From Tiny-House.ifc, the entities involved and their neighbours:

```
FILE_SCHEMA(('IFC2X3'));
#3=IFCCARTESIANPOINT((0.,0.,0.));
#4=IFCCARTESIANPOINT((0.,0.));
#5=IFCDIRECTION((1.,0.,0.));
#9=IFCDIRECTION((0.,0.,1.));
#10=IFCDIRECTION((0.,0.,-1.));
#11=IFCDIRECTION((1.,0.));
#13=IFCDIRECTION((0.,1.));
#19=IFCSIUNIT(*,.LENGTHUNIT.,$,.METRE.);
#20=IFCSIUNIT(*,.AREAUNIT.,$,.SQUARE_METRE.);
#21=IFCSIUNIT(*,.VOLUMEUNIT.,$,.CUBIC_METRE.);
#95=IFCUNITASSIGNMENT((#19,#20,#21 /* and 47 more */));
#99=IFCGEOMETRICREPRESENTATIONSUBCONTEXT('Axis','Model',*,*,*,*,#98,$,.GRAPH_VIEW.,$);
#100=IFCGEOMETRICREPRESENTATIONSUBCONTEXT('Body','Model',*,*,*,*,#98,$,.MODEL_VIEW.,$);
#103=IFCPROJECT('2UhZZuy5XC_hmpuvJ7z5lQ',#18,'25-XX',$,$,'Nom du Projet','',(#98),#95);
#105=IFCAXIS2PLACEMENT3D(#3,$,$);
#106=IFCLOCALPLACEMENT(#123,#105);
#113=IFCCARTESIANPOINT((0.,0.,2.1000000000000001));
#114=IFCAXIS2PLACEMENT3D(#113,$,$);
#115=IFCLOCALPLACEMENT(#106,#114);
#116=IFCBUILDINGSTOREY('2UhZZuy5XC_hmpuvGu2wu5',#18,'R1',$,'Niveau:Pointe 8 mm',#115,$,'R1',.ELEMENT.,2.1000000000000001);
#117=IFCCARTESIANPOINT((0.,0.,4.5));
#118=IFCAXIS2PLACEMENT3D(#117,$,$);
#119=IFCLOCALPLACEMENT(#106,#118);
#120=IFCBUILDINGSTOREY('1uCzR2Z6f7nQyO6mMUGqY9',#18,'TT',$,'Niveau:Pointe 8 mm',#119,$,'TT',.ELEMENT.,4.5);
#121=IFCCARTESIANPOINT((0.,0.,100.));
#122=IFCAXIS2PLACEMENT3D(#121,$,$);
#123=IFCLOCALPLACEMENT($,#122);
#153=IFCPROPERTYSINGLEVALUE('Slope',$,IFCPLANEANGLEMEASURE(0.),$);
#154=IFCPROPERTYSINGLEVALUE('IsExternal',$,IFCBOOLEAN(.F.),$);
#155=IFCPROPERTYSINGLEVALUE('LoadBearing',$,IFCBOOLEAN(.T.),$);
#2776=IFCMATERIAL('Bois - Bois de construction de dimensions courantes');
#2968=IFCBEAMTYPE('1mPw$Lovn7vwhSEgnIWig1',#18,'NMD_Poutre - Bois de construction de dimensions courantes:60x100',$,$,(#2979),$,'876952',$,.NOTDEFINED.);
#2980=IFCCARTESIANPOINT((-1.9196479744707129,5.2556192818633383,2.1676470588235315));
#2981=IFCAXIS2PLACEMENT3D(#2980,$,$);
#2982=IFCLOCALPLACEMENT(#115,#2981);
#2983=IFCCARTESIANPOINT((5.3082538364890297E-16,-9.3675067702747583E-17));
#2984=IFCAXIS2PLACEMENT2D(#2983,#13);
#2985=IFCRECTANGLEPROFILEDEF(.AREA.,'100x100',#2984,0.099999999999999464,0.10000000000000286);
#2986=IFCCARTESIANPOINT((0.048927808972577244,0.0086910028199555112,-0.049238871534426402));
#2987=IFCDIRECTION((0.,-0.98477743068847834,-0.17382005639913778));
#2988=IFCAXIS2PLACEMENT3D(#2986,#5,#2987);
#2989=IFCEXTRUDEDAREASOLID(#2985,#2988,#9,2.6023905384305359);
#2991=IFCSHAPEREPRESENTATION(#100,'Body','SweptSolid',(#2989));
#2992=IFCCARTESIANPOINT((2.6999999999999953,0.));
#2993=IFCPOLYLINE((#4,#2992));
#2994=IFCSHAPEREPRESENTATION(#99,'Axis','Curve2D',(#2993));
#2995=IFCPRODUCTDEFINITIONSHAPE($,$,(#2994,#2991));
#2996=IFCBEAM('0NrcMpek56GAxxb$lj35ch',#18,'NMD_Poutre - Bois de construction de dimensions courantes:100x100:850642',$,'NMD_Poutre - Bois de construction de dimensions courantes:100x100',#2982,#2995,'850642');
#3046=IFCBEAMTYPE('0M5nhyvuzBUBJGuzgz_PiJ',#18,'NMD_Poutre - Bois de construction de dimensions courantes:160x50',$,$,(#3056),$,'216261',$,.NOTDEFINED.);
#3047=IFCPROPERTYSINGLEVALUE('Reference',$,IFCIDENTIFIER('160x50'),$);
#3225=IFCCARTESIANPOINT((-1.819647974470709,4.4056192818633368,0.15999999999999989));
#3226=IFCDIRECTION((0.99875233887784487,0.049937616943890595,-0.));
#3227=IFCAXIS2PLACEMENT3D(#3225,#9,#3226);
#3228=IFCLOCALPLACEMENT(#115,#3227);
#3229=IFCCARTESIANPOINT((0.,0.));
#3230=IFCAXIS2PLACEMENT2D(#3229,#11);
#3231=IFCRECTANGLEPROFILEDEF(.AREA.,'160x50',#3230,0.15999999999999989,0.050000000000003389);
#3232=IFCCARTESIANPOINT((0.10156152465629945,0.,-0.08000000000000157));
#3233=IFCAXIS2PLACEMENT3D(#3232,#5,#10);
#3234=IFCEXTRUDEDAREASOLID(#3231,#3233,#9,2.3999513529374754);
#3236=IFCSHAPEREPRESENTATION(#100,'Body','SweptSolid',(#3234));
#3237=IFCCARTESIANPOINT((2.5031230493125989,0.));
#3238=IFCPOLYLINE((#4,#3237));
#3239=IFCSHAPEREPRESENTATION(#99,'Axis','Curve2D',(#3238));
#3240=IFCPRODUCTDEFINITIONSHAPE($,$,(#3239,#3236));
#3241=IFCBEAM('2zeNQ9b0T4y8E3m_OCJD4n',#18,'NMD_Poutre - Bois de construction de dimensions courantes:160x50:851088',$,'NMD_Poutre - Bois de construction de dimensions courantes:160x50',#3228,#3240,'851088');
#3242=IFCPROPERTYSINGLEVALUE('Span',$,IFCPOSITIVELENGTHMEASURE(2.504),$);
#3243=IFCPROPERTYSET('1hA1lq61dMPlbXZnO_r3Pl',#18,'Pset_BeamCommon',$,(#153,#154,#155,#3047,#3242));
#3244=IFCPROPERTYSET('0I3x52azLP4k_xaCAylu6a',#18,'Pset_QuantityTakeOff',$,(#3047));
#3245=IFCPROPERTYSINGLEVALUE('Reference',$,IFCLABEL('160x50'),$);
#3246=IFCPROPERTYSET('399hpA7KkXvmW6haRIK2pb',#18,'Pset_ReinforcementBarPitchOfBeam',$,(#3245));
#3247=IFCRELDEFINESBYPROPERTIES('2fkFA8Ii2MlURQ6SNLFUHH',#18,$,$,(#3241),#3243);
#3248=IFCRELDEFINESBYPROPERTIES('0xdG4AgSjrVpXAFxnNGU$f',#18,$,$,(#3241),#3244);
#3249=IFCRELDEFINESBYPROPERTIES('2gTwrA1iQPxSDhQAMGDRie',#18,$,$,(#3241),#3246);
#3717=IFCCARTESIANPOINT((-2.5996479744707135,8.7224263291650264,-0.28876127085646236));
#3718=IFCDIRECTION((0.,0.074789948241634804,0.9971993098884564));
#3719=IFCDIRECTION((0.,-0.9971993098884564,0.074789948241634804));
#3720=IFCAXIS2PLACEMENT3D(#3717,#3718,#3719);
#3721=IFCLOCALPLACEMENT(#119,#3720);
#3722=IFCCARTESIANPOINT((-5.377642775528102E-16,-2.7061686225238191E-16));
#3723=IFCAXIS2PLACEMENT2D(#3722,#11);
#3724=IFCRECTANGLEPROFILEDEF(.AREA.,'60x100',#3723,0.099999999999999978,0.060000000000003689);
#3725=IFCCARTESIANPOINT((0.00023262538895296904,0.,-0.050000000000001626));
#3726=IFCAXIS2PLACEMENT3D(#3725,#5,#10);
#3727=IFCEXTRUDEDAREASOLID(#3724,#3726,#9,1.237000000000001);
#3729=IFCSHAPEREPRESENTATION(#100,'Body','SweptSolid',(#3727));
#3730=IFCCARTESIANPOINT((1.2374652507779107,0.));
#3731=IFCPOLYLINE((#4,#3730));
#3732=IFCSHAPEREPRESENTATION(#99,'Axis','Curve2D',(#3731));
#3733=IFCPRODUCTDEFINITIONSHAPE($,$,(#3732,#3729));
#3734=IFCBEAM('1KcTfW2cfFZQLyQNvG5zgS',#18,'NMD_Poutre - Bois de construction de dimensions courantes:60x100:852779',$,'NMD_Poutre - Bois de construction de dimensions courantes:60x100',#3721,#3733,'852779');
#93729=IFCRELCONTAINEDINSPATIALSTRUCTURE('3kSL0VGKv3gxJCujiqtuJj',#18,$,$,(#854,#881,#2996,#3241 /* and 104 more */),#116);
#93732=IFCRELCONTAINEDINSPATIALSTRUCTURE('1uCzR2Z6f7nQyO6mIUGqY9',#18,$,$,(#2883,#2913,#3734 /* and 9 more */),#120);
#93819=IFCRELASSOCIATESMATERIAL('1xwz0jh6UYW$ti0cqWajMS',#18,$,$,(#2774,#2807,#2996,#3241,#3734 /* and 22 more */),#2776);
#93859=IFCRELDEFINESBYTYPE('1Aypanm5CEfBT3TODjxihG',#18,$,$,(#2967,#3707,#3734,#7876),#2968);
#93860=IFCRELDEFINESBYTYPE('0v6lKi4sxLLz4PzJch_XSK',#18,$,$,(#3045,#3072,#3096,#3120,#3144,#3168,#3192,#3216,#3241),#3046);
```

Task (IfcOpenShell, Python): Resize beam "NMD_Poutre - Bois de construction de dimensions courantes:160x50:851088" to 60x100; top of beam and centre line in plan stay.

```python
import ifcopenshell
import ifcopenshell.api.pset
import ifcopenshell.api.type
import ifcopenshell.util.element
import ifcopenshell.util.representation

model = ifcopenshell.open("Tiny-House.ifc")

member = model.by_guid("2zeNQ9b0T4y8E3m_OCJD4n")
source = next(p for p in model.by_type("IfcRectangleProfileDef") if p.ProfileName == "60x100")

body = ifcopenshell.util.representation.get_representation(member, "Model", "Body")
solid = body.Items[0]
old_profile = solid.SweptArea

# Copy the section's sizes but keep this member's own profile position.
profile = ifcopenshell.util.element.copy(model, source)
# Profiles are centred, so shift by half the change in depth to hold the top.
shift = (old_profile.XDim - profile.XDim) / 2
x, y = old_profile.Position.Location.Coordinates
up = (-1.0, 0.0)  # upwards, in the solid's own plane
location = model.createIfcCartesianPoint((x + up[0] * shift, y + up[1] * shift))
profile.Position = model.createIfcAxis2Placement2D(location, old_profile.Position.RefDirection)
solid.SweptArea = profile
if not model.get_total_inverses(old_profile):
    ifcopenshell.util.element.remove_deep2(model, old_profile)

new_type = model.by_guid("1mPw$Lovn7vwhSEgnIWig1")
ifcopenshell.api.type.assign_type(
    model, related_objects=[member], relating_type=new_type, should_map_representations=False
)
member.Name = member.Name.replace("160x50", "60x100")
member.ObjectType = "NMD_Poutre - Bois de construction de dimensions courantes:60x100"
pset = model.by_id(ifcopenshell.util.element.get_pset(member, "Pset_BeamCommon", should_inherit=False)["id"])
ifcopenshell.api.pset.edit_pset(model, pset=pset, properties={"Reference": "60x100"})
pset = model.by_id(ifcopenshell.util.element.get_pset(member, "Pset_QuantityTakeOff", should_inherit=False)["id"])
ifcopenshell.api.pset.edit_pset(model, pset=pset, properties={"Reference": "60x100"})
pset = model.by_id(ifcopenshell.util.element.get_pset(member, "Pset_ReinforcementBarPitchOfBeam", should_inherit=False)["id"])
ifcopenshell.api.pset.edit_pset(model, pset=pset, properties={"Reference": "60x100"})

print(solid.SweptArea)

model.write("Tiny-House_v2.ifc")
```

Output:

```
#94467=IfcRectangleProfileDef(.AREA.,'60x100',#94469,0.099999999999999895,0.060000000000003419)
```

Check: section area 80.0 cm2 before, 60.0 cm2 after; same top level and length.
